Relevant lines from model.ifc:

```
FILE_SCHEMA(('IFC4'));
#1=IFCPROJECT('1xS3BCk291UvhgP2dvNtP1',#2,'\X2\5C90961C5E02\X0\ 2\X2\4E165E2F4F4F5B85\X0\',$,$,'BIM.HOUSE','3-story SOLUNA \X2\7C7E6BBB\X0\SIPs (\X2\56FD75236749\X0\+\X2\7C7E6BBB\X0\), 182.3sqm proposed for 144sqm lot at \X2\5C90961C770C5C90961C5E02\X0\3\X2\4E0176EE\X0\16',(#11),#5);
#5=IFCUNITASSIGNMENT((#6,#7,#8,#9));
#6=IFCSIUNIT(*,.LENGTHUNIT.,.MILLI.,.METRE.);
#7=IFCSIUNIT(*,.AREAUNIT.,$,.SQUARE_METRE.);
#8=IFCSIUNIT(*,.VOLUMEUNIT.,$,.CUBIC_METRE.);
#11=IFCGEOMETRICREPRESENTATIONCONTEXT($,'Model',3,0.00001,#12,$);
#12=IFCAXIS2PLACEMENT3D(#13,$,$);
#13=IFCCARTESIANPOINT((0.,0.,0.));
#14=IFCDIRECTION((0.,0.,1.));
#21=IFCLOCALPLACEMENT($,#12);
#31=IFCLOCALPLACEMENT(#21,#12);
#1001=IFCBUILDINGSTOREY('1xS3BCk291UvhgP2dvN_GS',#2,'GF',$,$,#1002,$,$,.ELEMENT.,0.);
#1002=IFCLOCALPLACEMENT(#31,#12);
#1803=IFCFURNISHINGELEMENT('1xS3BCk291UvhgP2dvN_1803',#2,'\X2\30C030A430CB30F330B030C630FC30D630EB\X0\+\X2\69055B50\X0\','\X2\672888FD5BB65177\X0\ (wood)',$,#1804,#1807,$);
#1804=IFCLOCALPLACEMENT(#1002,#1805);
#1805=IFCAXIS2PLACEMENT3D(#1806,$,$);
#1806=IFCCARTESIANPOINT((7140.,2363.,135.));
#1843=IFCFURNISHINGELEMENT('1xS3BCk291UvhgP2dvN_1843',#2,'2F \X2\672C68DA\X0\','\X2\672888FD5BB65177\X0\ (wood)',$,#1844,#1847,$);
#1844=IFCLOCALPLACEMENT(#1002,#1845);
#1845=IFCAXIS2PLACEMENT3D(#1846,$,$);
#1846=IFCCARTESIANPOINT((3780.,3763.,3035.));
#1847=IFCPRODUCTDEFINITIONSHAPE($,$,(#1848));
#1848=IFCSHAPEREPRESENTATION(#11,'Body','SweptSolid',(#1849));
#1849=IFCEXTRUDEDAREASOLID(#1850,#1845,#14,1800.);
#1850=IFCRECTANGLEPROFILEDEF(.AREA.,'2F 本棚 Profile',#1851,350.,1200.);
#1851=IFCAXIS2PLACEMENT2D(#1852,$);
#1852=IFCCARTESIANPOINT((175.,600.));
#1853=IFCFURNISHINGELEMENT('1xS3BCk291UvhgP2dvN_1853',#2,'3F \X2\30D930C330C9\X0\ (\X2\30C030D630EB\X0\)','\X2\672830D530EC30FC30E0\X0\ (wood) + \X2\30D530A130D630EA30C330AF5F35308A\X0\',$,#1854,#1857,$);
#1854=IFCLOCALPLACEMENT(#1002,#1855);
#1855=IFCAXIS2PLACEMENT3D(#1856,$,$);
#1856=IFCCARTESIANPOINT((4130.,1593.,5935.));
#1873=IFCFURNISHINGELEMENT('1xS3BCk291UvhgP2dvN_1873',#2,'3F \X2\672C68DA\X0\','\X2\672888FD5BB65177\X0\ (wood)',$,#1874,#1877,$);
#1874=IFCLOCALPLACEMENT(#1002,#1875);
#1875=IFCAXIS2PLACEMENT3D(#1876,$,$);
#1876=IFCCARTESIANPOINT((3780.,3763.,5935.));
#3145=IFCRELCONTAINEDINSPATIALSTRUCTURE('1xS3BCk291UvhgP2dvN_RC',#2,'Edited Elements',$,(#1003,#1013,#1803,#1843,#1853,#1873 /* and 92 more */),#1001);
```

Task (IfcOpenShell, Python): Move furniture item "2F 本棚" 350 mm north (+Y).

```python
import ifcopenshell
import ifcopenshell.api.geometry
import ifcopenshell.util.placement
import ifcopenshell.util.unit

model = ifcopenshell.open("model.ifc")
unit_scale = ifcopenshell.util.unit.calculate_unit_scale(model)

item = model.by_id(1843)
matrix = ifcopenshell.util.placement.get_local_placement(item.ObjectPlacement)
matrix[1, 3] += 0.35 / unit_scale
ifcopenshell.api.geometry.edit_object_placement(model, product=item, matrix=matrix, is_si=False)

print(ifcopenshell.util.placement.get_local_placement(item.ObjectPlacement).round(3) + 0.0)

model.write("model-out.ifc")
```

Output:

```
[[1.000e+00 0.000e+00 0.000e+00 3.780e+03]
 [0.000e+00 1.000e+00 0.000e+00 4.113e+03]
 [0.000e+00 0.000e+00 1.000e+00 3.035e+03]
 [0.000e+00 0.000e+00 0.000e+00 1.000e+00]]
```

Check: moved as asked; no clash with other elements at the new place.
